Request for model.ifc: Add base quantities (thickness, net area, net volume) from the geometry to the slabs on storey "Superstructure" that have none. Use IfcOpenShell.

First a look at what the model holds.

```python
import ifcopenshell
import ifcopenshell.util.element
import ifcopenshell.util.unit

model = ifcopenshell.open("model.ifc")
print(model.schema)
for unit_type in ("LENGTHUNIT", "AREAUNIT", "VOLUMEUNIT"):
    print(unit_type, ifcopenshell.util.unit.calculate_unit_scale(model, unit_type))
storey = next(s for s in model.by_type("IfcBuildingStorey") if s.Name == "Superstructure")
slabs = [e for e in ifcopenshell.util.element.get_decomposition(storey) if e.is_a("IfcSlab")]
for e in sorted(slabs, key=lambda e: e.id()):
    print(e.id(), e.is_a(), e.Name, list(ifcopenshell.util.element.get_psets(e, qtos_only=True)), sep=" | ")
```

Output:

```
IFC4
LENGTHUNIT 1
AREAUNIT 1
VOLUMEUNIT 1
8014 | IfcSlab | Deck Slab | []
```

```python
import ifcopenshell
import ifcopenshell.api.pset
import ifcopenshell.geom
import ifcopenshell.util.element
import ifcopenshell.util.shape
import ifcopenshell.util.unit

model = ifcopenshell.open("model.ifc")
unit_scale = ifcopenshell.util.unit.calculate_unit_scale(model)
area_scale = ifcopenshell.util.unit.calculate_unit_scale(model, "AREAUNIT")
volume_scale = ifcopenshell.util.unit.calculate_unit_scale(model, "VOLUMEUNIT")
settings = ifcopenshell.geom.settings()

storey = next(s for s in model.by_type("IfcBuildingStorey") if s.Name == "Superstructure")
slabs = [e for e in ifcopenshell.util.element.get_decomposition(storey) if e.is_a("IfcSlab")]

for e in sorted(slabs, key=lambda e: e.id()):
    if ifcopenshell.util.element.get_psets(e, qtos_only=True, should_inherit=False):
        continue
    # Geometry comes back in metres, in the element's own axes.
    shape = ifcopenshell.geom.create_shape(settings, e)
    values = {
        "Width": ifcopenshell.util.shape.get_z(shape.geometry) / unit_scale,
        "NetArea": ifcopenshell.util.shape.get_footprint_area(shape.geometry) / area_scale,
        "NetVolume": ifcopenshell.util.shape.get_volume(shape.geometry) / volume_scale,
    }
    qto = ifcopenshell.api.pset.add_qto(model, product=e, name="Qto_SlabBaseQuantities")
    ifcopenshell.api.pset.edit_qto(model, qto=qto, properties=values)
    print(e.id(), {k: round(v, 3) for k, v in values.items()})

model.write("model_edited.ifc")
```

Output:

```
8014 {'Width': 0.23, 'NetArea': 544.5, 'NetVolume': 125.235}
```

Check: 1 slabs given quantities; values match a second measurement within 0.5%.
